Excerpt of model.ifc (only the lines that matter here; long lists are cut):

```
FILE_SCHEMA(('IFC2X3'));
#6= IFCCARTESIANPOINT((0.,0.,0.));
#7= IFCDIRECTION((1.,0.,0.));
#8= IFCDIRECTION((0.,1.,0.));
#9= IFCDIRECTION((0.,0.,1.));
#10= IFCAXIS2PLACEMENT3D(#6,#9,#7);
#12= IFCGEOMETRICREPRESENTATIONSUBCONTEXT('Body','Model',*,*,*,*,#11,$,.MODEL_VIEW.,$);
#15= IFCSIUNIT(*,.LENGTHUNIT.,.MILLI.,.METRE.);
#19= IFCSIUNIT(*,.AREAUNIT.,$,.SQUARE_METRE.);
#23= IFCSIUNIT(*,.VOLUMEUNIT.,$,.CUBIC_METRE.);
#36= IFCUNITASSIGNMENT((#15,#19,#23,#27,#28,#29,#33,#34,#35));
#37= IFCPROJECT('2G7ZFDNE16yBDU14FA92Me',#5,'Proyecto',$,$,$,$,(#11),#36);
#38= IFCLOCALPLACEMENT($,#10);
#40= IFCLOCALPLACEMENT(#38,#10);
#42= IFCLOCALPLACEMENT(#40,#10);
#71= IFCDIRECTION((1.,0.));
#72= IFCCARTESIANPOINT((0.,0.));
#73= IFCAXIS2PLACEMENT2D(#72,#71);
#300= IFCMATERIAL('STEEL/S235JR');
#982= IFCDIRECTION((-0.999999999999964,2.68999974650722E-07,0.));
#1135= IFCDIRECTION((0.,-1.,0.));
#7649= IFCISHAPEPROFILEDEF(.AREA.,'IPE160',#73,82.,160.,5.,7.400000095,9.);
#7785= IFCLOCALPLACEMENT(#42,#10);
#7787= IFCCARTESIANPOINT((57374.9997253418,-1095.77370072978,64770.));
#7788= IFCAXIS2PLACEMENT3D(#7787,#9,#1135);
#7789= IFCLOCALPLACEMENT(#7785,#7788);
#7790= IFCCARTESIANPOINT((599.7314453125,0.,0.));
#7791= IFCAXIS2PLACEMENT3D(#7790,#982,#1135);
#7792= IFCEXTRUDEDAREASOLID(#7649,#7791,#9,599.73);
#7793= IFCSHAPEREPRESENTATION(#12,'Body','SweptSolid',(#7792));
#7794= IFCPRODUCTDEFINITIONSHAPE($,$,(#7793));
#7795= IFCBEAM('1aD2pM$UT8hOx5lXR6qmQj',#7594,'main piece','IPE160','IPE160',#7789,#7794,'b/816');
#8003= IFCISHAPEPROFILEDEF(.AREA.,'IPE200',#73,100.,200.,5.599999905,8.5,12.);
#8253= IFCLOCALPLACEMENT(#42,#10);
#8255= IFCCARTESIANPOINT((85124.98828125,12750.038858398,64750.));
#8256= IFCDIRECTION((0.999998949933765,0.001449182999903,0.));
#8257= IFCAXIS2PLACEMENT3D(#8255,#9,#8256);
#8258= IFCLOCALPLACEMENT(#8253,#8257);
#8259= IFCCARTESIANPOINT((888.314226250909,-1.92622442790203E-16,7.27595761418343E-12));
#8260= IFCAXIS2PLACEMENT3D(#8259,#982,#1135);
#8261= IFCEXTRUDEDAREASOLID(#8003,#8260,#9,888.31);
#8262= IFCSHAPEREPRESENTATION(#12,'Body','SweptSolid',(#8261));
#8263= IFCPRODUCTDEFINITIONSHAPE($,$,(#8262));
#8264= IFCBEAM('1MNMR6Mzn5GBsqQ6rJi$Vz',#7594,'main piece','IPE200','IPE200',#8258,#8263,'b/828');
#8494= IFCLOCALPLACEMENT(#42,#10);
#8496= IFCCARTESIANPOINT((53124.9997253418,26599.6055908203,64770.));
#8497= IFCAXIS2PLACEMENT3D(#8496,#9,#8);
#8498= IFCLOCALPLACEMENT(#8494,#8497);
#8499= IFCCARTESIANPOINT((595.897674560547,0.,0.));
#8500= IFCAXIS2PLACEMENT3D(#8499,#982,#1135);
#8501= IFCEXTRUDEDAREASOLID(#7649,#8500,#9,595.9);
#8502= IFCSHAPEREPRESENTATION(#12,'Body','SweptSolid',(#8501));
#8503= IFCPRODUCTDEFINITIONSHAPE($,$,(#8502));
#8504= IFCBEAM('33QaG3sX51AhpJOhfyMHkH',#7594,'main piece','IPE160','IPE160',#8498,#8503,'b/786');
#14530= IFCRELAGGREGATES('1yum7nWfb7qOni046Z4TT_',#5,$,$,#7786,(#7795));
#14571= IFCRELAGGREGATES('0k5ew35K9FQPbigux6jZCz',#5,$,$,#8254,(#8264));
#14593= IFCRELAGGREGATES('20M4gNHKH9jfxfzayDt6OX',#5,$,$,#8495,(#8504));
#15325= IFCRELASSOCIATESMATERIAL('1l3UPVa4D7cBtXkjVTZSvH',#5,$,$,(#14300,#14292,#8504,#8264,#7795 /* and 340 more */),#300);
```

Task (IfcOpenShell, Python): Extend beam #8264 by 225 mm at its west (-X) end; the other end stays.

```python
import ifcopenshell
import ifcopenshell.util.representation

model = ifcopenshell.open("model.ifc")

member = model.by_guid("1MNMR6Mzn5GBsqQ6rJi$Vz")
change = 225.0

# The extrusion runs towards the end named, so only its depth changes.
body = ifcopenshell.util.representation.get_representation(member, "Model", "Body")
solid = body.Items[0]
old_length = solid.Depth
solid.Depth += change

print(f"length {old_length:g} -> {solid.Depth:g}")

model.write("model_v2.ifc")
```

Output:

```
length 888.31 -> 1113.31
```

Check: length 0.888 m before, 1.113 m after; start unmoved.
